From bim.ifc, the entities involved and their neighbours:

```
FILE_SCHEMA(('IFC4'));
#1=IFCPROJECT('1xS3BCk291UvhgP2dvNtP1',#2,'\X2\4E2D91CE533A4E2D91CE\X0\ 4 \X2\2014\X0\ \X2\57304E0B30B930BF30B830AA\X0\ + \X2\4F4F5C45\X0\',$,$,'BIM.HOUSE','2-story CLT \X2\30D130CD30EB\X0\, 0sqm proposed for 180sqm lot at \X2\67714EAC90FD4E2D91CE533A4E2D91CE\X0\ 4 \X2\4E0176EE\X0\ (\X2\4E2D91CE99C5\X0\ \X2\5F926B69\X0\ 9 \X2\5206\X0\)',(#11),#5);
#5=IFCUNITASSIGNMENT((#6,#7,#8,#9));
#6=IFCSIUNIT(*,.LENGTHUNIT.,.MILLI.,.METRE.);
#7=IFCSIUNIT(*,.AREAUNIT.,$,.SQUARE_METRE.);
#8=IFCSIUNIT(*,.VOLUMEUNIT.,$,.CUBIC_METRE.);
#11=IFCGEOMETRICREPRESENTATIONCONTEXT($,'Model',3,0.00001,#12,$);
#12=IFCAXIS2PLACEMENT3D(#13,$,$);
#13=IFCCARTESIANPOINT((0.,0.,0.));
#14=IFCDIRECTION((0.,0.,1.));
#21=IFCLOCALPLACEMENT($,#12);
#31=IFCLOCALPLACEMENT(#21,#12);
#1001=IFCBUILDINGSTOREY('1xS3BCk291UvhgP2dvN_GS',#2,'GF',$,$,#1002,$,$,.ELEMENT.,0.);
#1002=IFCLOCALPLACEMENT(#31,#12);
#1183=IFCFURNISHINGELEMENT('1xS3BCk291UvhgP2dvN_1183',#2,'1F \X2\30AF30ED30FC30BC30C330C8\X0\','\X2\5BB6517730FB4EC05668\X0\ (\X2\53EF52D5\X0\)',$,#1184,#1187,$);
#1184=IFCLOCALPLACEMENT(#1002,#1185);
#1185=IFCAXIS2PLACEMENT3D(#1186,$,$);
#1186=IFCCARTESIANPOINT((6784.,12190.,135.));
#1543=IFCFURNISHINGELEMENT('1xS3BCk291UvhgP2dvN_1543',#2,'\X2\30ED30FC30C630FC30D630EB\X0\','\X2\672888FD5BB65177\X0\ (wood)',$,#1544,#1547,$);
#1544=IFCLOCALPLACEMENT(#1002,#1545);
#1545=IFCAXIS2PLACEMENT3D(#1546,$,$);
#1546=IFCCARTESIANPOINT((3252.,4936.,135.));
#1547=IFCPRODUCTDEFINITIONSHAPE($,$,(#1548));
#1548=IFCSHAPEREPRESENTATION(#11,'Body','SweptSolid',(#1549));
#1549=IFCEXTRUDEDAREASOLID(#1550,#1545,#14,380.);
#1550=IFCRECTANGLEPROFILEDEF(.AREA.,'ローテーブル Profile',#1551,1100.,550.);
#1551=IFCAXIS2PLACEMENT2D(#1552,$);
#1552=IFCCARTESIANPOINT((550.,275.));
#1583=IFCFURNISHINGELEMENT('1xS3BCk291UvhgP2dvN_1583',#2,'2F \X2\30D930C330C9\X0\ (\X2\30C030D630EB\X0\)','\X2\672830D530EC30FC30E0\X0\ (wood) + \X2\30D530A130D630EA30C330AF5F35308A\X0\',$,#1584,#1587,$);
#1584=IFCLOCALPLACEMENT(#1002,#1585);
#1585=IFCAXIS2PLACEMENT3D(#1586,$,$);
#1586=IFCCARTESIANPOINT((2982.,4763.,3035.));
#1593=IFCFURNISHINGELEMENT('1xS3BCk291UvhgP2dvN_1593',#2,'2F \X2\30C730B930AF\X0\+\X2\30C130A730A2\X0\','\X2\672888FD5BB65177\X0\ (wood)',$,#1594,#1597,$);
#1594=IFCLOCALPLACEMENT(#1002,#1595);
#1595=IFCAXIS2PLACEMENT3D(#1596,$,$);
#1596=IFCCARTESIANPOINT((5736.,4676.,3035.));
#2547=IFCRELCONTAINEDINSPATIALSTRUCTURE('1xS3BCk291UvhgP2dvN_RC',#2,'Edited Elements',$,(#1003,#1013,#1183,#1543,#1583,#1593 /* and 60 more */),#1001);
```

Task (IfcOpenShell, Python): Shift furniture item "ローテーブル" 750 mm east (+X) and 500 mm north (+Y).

```python
import ifcopenshell
import ifcopenshell.api.geometry
import ifcopenshell.util.placement
import ifcopenshell.util.unit

model = ifcopenshell.open("bim.ifc")
unit_scale = ifcopenshell.util.unit.calculate_unit_scale(model)

item = model.by_guid("1xS3BCk291UvhgP2dvN_1543")
matrix = ifcopenshell.util.placement.get_local_placement(item.ObjectPlacement)
matrix[0, 3] += 0.75 / unit_scale
matrix[1, 3] += 0.5 / unit_scale
ifcopenshell.api.geometry.edit_object_placement(model, product=item, matrix=matrix, is_si=False)

print(ifcopenshell.util.placement.get_local_placement(item.ObjectPlacement).round(3) + 0.0)

model.write("bim_updated.ifc")
```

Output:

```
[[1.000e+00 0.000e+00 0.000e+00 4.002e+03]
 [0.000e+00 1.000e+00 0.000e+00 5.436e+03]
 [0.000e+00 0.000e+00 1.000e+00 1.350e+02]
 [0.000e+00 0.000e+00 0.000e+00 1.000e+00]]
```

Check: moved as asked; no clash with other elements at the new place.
